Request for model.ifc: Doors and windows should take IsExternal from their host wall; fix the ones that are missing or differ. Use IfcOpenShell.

First a look at what the model holds.

```python
import ifcopenshell
import ifcopenshell.util.element

model = ifcopenshell.open("model.ifc")
print(model.schema)
seen = {}
for e in model.by_type("IfcDoor") + model.by_type("IfcWindow"):
    if not e.FillsVoids:
        continue
    host = e.FillsVoids[0].RelatingOpeningElement.VoidsElements[0].RelatingBuildingElement
    own = ifcopenshell.util.element.get_pset(e, f"Pset_{e.is_a()[3:].removesuffix('StandardCase')}Common", "IsExternal")
    wall = ifcopenshell.util.element.get_pset(host, "Pset_WallCommon", "IsExternal")
    seen[e.is_a(), own, wall] = seen.get((e.is_a(), own, wall), 0) + 1
for (cls, own, wall), count in sorted(seen.items(), key=str):
    print(count, cls, "IsExternal:", own, "| host wall:", wall)
```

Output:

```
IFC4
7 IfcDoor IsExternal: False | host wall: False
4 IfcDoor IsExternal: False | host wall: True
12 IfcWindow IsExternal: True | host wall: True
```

```python
import ifcopenshell
import ifcopenshell.api.pset
import ifcopenshell.util.element

model = ifcopenshell.open("model.ifc")

count = 0
for ifc_class, pset_name in (("IfcDoor", "Pset_DoorCommon"), ("IfcWindow", "Pset_WindowCommon")):
    for e in model.by_type(ifc_class):
        if not e.FillsVoids:
            continue
        host = e.FillsVoids[0].RelatingOpeningElement.VoidsElements[0].RelatingBuildingElement
        external = ifcopenshell.util.element.get_pset(host, "Pset_WallCommon", "IsExternal")
        if external is None or ifcopenshell.util.element.get_pset(e, pset_name, "IsExternal") == external:
            continue
        pset = ifcopenshell.api.pset.add_pset(model, product=e, name=pset_name)
        ifcopenshell.api.pset.edit_pset(model, pset=pset, properties={"IsExternal": external})
        count += 1

print(count, "updated")

model.write("model_edited.ifc")
```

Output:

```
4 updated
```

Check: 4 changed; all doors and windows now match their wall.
